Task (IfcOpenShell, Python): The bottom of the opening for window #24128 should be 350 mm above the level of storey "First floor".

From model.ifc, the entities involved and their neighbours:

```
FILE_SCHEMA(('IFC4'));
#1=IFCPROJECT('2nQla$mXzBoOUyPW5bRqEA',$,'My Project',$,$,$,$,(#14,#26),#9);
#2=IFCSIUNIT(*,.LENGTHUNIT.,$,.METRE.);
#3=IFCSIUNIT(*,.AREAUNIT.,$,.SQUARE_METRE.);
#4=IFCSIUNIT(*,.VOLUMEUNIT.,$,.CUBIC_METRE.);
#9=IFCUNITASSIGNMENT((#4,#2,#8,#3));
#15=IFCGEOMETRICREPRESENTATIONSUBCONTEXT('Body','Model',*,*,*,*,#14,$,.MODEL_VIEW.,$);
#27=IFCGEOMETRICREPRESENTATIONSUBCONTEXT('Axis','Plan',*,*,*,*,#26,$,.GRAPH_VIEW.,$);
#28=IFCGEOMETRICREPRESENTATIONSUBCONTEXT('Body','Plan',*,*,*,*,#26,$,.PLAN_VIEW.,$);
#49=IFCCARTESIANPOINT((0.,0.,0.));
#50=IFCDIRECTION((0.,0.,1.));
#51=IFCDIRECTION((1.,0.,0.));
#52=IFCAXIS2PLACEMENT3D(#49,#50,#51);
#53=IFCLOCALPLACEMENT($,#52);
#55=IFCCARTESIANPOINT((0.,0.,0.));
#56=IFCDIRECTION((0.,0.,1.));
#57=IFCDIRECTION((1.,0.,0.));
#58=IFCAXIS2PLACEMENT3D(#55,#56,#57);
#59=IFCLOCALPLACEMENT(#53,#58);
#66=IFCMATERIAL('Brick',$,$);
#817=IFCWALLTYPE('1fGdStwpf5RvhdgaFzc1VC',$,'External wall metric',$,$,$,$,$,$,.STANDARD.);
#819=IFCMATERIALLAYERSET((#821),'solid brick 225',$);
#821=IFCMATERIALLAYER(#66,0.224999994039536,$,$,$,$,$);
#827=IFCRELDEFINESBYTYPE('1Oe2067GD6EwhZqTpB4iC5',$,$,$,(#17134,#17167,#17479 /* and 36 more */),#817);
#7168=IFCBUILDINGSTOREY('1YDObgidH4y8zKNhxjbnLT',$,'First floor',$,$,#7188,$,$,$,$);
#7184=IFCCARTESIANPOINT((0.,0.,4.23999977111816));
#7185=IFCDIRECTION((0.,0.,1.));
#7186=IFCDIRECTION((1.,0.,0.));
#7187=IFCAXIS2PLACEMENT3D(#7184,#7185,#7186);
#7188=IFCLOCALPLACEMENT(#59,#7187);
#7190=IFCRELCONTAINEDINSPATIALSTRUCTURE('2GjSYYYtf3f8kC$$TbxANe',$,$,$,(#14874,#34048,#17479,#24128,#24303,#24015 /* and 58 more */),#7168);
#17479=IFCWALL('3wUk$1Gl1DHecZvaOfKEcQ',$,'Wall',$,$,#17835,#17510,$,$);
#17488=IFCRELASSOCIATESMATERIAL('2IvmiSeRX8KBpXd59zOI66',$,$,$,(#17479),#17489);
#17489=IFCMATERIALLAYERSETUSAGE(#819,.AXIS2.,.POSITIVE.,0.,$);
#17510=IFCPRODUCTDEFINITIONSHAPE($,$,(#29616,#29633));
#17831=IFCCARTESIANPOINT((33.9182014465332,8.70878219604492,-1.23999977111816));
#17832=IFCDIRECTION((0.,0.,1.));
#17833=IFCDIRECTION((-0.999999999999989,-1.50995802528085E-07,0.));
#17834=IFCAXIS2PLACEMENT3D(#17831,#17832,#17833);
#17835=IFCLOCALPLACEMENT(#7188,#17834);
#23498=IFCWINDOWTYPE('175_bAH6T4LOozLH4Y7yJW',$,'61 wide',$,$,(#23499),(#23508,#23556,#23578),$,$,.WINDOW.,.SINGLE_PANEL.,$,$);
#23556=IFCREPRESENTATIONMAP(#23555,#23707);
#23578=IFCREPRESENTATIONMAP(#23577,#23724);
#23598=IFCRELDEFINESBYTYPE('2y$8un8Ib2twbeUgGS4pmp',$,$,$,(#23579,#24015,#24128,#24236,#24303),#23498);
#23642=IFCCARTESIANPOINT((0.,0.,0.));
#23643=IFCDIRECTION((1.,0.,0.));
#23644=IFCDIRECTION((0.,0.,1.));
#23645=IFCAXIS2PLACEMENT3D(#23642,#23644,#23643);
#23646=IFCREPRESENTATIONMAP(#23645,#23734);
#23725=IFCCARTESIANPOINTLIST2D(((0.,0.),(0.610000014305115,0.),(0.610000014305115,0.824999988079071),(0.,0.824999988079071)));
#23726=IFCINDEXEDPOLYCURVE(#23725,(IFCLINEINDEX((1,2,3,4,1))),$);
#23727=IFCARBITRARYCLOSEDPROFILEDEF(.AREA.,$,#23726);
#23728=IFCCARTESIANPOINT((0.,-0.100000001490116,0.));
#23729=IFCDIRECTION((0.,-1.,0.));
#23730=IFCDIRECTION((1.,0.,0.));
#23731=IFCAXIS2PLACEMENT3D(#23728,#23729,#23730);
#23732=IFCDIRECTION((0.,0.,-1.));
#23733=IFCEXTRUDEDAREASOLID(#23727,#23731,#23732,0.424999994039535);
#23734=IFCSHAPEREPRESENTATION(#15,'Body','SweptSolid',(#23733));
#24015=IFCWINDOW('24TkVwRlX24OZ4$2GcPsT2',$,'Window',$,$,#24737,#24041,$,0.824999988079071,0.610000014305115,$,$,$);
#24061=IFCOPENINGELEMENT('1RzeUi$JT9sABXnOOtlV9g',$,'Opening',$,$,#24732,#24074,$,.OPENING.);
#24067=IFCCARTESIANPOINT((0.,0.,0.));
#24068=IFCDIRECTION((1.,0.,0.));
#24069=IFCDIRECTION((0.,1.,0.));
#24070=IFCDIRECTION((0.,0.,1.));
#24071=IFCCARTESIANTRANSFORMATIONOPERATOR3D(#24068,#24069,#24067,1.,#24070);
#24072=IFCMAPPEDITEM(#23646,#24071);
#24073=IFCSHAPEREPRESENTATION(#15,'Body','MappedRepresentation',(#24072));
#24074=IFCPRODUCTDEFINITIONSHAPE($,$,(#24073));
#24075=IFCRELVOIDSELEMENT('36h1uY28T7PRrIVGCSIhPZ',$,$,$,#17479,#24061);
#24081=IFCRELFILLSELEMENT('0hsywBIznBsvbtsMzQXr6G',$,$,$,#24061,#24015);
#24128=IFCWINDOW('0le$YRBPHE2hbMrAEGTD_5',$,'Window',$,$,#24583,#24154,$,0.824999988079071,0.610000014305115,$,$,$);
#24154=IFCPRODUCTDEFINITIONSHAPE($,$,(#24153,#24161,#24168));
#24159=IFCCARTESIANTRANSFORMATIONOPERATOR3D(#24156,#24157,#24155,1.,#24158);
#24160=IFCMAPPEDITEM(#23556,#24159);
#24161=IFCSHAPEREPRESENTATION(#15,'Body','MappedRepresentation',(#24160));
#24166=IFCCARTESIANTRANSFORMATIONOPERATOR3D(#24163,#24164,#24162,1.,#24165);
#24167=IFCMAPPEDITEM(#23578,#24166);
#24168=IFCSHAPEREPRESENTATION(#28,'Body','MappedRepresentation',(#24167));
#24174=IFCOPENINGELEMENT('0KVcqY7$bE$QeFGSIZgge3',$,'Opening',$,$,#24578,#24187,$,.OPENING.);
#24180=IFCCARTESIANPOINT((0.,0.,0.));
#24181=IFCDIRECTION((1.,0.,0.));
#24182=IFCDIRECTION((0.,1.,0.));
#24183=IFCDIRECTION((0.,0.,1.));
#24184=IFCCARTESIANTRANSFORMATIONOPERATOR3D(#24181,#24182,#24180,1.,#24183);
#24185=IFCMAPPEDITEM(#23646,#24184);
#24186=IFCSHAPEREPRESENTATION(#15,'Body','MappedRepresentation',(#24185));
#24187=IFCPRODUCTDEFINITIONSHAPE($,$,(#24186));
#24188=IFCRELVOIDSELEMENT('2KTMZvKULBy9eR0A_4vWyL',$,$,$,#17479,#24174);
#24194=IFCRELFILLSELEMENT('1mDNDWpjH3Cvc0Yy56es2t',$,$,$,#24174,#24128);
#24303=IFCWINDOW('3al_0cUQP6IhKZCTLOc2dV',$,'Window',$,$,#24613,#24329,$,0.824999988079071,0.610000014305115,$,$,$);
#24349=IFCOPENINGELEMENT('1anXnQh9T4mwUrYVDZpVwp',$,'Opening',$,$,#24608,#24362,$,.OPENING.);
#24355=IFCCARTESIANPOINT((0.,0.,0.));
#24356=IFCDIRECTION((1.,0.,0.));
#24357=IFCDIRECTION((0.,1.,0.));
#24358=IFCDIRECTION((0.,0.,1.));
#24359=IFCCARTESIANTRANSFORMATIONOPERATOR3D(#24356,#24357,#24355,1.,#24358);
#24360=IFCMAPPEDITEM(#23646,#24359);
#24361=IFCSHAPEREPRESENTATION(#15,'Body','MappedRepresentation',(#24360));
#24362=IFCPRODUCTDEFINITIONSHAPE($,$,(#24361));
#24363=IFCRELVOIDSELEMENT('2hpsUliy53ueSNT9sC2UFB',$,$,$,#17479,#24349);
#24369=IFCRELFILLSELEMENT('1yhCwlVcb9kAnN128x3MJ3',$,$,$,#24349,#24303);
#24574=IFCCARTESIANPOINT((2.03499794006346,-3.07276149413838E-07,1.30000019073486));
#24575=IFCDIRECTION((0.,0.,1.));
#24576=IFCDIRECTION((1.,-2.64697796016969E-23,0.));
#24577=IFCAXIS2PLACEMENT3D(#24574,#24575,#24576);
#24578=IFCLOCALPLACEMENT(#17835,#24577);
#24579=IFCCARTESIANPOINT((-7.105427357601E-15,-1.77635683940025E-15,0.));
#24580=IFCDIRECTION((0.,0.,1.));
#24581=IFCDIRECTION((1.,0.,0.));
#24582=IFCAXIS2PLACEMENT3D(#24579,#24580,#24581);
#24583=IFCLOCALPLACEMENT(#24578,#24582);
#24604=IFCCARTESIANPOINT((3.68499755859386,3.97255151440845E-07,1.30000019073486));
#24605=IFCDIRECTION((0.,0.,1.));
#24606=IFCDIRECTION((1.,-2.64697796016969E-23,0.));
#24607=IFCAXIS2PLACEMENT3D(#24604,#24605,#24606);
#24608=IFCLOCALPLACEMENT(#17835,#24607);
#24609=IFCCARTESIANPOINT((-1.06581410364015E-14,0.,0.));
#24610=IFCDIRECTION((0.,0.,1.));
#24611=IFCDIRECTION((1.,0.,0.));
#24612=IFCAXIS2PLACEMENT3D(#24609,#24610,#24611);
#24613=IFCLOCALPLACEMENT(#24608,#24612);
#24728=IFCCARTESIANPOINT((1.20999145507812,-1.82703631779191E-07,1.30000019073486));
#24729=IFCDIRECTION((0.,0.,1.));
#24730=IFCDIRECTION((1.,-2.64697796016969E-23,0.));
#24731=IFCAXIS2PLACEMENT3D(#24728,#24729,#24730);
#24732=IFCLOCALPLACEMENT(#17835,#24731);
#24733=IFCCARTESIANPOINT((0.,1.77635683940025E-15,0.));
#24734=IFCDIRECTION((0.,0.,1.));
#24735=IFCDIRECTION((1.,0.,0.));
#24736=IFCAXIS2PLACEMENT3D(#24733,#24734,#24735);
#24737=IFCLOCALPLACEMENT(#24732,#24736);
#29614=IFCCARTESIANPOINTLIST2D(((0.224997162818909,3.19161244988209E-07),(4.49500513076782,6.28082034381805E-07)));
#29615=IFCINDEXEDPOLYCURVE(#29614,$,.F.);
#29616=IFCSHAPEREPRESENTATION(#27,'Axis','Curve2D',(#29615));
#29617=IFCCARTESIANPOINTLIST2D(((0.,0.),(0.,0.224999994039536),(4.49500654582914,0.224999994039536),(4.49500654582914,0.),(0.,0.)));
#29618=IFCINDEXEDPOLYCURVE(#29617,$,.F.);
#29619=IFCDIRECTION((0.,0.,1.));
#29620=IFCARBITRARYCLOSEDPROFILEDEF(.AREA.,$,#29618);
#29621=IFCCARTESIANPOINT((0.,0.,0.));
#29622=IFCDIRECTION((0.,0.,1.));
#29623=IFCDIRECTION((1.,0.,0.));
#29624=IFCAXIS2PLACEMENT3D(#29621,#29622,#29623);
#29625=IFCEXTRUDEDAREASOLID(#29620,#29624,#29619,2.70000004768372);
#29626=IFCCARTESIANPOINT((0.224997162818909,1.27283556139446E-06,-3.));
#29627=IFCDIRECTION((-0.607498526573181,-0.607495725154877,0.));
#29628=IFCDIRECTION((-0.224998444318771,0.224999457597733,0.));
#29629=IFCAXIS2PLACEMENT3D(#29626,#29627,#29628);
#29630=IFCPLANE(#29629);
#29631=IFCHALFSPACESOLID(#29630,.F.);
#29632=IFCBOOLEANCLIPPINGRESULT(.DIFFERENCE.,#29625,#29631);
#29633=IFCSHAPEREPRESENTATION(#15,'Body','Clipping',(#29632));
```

```python
import numpy as np
import ifcopenshell
import ifcopenshell.api.geometry
import ifcopenshell.geom
import ifcopenshell.util.element
import ifcopenshell.util.placement
import ifcopenshell.util.shape
import ifcopenshell.util.unit

model = ifcopenshell.open("model.ifc")
unit_scale = ifcopenshell.util.unit.calculate_unit_scale(model)

window = model.by_id(24128)
opening = window.FillsVoids[0].RelatingOpeningElement
storey = ifcopenshell.util.element.get_container(window, ifc_class="IfcBuildingStorey")
level = ifcopenshell.util.placement.get_local_placement(storey.ObjectPlacement)[2, 3]

# The opening's origin need not be at the sill, so measure its lowest point.
shape = ifcopenshell.geom.create_shape(ifcopenshell.geom.settings(), opening)
bottom = ifcopenshell.util.shape.get_shape_bottom_elevation(shape, shape.geometry) / unit_scale
dz = level + 0.35 - bottom

shift = np.array([0.0, 0.0, dz])
# The window is placed relative to its opening, so it follows when the opening moves.
matrix = ifcopenshell.util.placement.get_local_placement(opening.ObjectPlacement)
matrix[:3, 3] += shift
ifcopenshell.api.geometry.edit_object_placement(
    model, product=opening, matrix=matrix, is_si=False, should_transform_children=True
)

print(f"moved by {dz * unit_scale:+.3f} m")

model.write("model_updated.ifc")
```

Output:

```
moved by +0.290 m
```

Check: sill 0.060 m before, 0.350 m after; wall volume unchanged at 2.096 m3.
